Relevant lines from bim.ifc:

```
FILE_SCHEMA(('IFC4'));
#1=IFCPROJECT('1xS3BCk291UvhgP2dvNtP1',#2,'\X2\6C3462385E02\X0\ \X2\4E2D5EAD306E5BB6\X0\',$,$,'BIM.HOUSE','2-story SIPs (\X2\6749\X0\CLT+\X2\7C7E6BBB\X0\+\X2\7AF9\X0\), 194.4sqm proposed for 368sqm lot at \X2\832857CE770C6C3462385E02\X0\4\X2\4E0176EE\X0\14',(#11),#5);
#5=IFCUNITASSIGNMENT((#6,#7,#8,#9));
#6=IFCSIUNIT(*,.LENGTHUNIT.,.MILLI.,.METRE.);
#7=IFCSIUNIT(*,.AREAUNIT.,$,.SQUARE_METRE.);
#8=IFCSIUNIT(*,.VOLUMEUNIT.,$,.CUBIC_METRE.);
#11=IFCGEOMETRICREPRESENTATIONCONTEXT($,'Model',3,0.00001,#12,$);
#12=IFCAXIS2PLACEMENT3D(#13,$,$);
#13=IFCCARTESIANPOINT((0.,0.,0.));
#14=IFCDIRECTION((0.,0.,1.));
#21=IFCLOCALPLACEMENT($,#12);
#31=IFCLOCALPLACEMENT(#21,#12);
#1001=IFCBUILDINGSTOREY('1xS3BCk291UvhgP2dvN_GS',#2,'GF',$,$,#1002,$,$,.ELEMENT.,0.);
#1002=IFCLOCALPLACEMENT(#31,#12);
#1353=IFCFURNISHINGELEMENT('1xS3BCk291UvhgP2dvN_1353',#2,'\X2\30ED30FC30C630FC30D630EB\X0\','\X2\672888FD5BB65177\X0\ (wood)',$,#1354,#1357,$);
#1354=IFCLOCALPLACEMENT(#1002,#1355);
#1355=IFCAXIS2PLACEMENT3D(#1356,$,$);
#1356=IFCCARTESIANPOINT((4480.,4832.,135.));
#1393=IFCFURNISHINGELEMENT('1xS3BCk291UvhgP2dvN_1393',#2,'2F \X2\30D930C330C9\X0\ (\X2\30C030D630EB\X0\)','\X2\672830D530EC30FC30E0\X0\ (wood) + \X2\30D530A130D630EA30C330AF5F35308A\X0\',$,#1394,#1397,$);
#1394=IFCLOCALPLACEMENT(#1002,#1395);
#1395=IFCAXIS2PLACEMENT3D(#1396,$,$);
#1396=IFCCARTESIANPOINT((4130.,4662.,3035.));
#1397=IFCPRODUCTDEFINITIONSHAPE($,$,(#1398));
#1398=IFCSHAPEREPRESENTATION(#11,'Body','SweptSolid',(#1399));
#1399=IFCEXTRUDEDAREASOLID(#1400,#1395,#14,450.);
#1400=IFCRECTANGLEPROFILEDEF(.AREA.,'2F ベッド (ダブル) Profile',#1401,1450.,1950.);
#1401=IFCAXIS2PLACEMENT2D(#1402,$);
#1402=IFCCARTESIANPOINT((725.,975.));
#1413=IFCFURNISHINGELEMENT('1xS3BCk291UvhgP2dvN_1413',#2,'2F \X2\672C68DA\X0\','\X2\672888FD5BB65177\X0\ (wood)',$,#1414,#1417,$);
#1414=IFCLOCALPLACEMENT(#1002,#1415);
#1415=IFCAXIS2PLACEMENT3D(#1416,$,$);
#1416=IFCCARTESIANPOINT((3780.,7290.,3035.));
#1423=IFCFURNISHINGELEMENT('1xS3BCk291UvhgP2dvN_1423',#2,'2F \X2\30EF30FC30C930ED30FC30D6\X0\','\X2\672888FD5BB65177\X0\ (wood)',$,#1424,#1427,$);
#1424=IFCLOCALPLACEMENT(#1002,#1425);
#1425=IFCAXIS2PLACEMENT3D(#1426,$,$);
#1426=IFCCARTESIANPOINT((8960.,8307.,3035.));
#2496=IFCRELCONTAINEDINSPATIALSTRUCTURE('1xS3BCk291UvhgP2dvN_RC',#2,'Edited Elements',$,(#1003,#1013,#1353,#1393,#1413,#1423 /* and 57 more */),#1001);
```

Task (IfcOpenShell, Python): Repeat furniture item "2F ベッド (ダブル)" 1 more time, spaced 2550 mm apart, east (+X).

```python
import numpy as np
import ifcopenshell
import ifcopenshell.api.geometry
import ifcopenshell.api.root
import ifcopenshell.util.element
import ifcopenshell.util.placement
import ifcopenshell.util.unit

model = ifcopenshell.open("bim.ifc")
unit_scale = ifcopenshell.util.unit.calculate_unit_scale(model)


def reuse_history(source, copy):
    """copy_class also copies each property set's owner history, people and application; keep the originals."""
    for rel in copy.IsDefinedBy:
        if rel.is_a("IfcRelDefinesByProperties") and (history := rel.RelatingPropertyDefinition.OwnerHistory):
            rel.RelatingPropertyDefinition.OwnerHistory = source.OwnerHistory
            ifcopenshell.util.element.remove_deep2(model, history)


source = model.by_id(1393)
base = ifcopenshell.util.placement.get_local_placement(source.ObjectPlacement)
step = np.array([1.0, 0.0, 0.0]) * 2.55 / unit_scale

for i in range(1, 2):
    copy = ifcopenshell.api.root.copy_class(model, product=source)
    copy.Representation = ifcopenshell.util.element.copy_deep(
        model, source.Representation, exclude=["IfcGeometricRepresentationContext", "IfcRepresentationMap"]
    )
    reuse_history(source, copy)
    matrix = base.copy()
    matrix[:3, 3] += i * step
    print("added at", matrix[:3, 3].round(3) + 0.0)
    ifcopenshell.api.geometry.edit_object_placement(model, product=copy, matrix=matrix, is_si=False)

model.write("bim_edited.ifc")
```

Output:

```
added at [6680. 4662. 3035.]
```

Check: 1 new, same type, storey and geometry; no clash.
